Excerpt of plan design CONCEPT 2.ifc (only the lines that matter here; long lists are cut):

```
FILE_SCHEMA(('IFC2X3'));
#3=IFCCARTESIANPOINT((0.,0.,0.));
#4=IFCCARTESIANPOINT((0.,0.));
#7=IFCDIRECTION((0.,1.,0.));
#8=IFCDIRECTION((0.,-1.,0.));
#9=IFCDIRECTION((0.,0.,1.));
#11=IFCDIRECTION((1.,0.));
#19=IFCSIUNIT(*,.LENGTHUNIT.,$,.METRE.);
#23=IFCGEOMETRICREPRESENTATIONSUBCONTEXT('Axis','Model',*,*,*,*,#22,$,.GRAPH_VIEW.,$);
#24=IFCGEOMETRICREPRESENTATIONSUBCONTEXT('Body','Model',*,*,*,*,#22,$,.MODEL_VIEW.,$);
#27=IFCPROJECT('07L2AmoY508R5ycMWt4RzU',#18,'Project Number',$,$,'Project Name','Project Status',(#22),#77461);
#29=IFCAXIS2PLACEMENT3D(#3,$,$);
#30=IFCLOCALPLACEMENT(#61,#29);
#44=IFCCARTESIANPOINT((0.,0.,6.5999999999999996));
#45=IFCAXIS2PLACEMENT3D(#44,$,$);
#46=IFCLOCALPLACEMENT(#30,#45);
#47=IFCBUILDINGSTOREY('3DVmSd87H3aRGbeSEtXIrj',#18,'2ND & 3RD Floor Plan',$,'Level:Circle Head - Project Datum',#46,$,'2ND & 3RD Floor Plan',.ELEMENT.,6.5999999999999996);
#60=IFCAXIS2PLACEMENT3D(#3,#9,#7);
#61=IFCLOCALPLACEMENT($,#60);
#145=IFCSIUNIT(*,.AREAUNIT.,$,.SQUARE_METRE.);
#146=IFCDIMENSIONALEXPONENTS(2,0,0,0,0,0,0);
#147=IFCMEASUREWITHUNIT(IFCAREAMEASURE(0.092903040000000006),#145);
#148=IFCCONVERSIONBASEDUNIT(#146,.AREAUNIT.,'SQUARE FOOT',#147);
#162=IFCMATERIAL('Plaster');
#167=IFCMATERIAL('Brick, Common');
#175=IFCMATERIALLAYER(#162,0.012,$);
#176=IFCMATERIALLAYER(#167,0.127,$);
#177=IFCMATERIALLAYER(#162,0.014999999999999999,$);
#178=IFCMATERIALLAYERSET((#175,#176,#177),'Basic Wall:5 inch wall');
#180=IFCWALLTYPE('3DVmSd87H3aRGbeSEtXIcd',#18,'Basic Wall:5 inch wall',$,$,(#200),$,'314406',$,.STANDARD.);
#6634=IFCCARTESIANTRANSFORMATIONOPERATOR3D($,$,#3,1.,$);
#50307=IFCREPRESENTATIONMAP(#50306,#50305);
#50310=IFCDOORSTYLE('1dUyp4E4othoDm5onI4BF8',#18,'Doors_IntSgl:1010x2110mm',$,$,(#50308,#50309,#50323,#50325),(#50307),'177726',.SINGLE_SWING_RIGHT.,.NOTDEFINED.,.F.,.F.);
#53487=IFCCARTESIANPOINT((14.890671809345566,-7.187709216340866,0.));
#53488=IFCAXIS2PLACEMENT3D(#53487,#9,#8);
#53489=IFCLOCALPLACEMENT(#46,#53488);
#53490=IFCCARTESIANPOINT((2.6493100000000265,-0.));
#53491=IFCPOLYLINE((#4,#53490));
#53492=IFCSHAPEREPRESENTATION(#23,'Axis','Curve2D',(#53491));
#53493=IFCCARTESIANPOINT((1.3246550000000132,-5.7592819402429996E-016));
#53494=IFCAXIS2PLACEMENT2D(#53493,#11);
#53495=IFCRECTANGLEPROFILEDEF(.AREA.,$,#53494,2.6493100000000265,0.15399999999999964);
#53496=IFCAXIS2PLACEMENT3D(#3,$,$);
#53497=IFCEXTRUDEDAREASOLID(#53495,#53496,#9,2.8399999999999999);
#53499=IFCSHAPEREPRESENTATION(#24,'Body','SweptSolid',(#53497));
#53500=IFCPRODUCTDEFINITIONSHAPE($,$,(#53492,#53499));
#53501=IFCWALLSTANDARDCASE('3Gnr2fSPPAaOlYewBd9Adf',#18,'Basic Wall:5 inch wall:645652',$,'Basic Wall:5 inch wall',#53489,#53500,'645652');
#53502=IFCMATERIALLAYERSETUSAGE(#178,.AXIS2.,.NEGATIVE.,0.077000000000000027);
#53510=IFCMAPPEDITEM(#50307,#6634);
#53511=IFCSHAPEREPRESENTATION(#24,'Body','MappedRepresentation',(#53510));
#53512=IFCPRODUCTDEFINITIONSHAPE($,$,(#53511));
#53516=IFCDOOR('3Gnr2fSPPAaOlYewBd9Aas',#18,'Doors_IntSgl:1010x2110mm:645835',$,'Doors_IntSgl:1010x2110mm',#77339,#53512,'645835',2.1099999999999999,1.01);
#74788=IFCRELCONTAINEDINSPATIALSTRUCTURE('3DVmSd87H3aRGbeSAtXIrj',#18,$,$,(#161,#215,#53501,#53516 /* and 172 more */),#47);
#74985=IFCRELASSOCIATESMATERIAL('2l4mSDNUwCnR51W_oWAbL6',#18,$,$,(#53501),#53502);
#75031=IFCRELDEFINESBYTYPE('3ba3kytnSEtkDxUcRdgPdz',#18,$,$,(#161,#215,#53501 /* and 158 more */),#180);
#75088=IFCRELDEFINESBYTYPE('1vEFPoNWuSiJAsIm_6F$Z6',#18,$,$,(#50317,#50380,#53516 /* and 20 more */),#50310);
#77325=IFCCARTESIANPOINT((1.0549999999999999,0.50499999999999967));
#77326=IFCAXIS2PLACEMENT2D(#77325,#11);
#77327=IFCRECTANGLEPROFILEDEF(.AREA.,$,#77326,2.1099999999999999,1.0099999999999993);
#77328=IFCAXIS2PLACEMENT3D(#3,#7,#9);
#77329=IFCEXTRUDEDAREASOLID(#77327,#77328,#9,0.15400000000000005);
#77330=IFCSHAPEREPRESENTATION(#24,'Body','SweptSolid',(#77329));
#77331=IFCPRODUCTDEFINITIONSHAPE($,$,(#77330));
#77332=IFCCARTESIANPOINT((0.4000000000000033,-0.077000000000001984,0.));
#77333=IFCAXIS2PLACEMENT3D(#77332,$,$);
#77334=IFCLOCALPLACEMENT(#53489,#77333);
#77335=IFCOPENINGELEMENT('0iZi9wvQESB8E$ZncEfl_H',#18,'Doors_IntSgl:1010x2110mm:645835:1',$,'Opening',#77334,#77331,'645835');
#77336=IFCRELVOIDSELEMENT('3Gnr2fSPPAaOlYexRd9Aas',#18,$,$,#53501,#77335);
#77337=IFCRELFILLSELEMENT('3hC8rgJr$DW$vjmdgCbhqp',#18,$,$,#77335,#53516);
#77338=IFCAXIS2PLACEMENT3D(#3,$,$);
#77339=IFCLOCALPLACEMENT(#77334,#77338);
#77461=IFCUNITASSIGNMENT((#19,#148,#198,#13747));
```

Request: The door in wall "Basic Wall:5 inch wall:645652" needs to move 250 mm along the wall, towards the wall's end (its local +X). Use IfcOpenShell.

```python
import ifcopenshell
import ifcopenshell.api.geometry
import ifcopenshell.util.placement

model = ifcopenshell.open("plan design CONCEPT 2.ifc")

door = model.by_id(53516)
opening = door.FillsVoids[0].RelatingOpeningElement
wall = opening.VoidsElements[0].RelatingBuildingElement

wall_matrix = ifcopenshell.util.placement.get_local_placement(wall.ObjectPlacement)
shift = wall_matrix[:3, 0] * 0.25
before = ifcopenshell.util.placement.get_local_placement(door.ObjectPlacement)[:3, 3].copy()

# The door is placed relative to its opening, so it follows when the opening moves.
matrix = ifcopenshell.util.placement.get_local_placement(opening.ObjectPlacement)
matrix[:3, 3] += shift
ifcopenshell.api.geometry.edit_object_placement(
    model, product=opening, matrix=matrix, is_si=False, should_transform_children=True
)

after = ifcopenshell.util.placement.get_local_placement(door.ObjectPlacement)[:3, 3]
print("door moved by", (after - before).round(3) + 0.0)

model.write("plan design CONCEPT 2-out.ifc")
```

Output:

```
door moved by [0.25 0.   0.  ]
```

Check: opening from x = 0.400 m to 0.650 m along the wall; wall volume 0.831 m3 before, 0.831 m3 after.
